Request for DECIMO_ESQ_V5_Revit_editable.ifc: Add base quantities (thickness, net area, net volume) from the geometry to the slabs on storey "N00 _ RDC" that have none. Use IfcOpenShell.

First a look at what the model holds.

```python
import ifcopenshell
import ifcopenshell.util.element
import ifcopenshell.util.unit

model = ifcopenshell.open("DECIMO_ESQ_V5_Revit_editable.ifc")
print(model.schema)
for unit_type in ("LENGTHUNIT", "AREAUNIT", "VOLUMEUNIT"):
    print(unit_type, ifcopenshell.util.unit.calculate_unit_scale(model, unit_type))
storey = next(s for s in model.by_type("IfcBuildingStorey") if s.Name == "N00 _ RDC")
slabs = [e for e in ifcopenshell.util.element.get_decomposition(storey) if e.is_a("IfcSlab")]
for e in sorted(slabs, key=lambda e: e.id()):
    print(e.id(), e.is_a(), e.Name, list(ifcopenshell.util.element.get_psets(e, qtos_only=True)), sep=" | ")
```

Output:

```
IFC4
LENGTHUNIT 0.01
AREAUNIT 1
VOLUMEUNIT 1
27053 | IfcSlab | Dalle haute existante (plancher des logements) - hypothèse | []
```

```python
import ifcopenshell
import ifcopenshell.api.pset
import ifcopenshell.geom
import ifcopenshell.util.element
import ifcopenshell.util.shape
import ifcopenshell.util.unit

model = ifcopenshell.open("DECIMO_ESQ_V5_Revit_editable.ifc")
unit_scale = ifcopenshell.util.unit.calculate_unit_scale(model)
area_scale = ifcopenshell.util.unit.calculate_unit_scale(model, "AREAUNIT")
volume_scale = ifcopenshell.util.unit.calculate_unit_scale(model, "VOLUMEUNIT")
settings = ifcopenshell.geom.settings()

storey = next(s for s in model.by_type("IfcBuildingStorey") if s.Name == "N00 _ RDC")
slabs = [e for e in ifcopenshell.util.element.get_decomposition(storey) if e.is_a("IfcSlab")]

for e in sorted(slabs, key=lambda e: e.id()):
    if ifcopenshell.util.element.get_psets(e, qtos_only=True, should_inherit=False):
        continue
    # Geometry comes back in metres, in the element's own axes.
    shape = ifcopenshell.geom.create_shape(settings, e)
    values = {
        "Width": ifcopenshell.util.shape.get_z(shape.geometry) / unit_scale,
        "NetArea": ifcopenshell.util.shape.get_footprint_area(shape.geometry) / area_scale,
        "NetVolume": ifcopenshell.util.shape.get_volume(shape.geometry) / volume_scale,
    }
    qto = ifcopenshell.api.pset.add_qto(model, product=e, name="Qto_SlabBaseQuantities")
    ifcopenshell.api.pset.edit_qto(model, qto=qto, properties=values)
    print(e.id(), {k: round(v, 3) for k, v in values.items()})

model.write("DECIMO_ESQ_V5_Revit_editable_edited.ifc")
```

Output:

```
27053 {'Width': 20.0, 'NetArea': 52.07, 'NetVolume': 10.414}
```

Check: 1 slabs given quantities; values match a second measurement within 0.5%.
